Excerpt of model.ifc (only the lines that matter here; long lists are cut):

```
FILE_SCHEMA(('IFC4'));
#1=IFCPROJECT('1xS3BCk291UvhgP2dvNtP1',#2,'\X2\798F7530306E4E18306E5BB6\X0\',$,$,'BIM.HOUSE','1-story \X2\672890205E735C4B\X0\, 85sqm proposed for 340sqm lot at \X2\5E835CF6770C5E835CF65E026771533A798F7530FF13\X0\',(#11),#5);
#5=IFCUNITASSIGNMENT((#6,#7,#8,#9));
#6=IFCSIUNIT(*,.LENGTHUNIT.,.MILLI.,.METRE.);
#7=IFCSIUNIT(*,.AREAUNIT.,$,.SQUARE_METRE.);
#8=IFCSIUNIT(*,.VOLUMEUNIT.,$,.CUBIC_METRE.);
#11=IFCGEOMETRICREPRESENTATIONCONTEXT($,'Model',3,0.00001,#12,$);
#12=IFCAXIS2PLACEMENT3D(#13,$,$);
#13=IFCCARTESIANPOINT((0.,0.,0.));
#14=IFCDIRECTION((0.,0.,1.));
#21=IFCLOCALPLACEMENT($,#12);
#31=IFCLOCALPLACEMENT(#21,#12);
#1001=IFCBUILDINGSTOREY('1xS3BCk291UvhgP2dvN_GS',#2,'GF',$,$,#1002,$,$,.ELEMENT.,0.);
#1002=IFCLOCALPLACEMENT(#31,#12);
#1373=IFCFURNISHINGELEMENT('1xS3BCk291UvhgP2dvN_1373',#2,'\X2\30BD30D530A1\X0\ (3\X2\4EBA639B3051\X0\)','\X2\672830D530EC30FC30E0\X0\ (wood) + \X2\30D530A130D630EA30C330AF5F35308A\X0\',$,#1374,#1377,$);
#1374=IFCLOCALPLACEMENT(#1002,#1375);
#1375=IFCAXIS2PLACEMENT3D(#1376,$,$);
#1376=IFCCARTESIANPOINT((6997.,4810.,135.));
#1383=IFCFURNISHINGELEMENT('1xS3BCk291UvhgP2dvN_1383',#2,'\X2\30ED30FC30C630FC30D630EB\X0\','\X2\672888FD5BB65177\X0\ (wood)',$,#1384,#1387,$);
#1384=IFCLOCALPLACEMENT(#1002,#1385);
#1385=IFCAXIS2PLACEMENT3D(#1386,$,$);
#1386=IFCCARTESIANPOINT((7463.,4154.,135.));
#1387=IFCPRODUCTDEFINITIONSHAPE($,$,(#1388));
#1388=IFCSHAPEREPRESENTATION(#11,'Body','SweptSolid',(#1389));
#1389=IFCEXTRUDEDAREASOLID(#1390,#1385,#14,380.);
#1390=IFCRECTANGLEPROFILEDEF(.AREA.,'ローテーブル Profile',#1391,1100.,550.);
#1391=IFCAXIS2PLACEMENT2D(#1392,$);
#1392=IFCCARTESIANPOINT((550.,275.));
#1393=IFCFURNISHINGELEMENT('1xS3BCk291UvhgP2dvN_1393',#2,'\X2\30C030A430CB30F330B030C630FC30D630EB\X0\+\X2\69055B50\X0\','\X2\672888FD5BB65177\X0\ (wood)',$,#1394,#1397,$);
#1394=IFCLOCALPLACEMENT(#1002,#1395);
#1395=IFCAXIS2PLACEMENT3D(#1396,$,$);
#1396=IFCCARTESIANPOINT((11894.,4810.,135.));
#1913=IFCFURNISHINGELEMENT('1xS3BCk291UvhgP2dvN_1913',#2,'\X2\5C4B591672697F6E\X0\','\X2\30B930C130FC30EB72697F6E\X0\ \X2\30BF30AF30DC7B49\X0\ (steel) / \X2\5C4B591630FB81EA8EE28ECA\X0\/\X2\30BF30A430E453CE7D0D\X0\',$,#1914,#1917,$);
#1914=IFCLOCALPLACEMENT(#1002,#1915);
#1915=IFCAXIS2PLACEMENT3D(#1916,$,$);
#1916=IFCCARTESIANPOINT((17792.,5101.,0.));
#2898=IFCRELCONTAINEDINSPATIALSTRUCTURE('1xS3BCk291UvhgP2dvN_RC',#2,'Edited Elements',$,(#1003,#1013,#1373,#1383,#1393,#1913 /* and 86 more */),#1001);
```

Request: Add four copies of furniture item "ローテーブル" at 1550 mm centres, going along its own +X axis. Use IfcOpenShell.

```python
import ifcopenshell
import ifcopenshell.api.geometry
import ifcopenshell.api.root
import ifcopenshell.util.element
import ifcopenshell.util.placement
import ifcopenshell.util.unit

model = ifcopenshell.open("model.ifc")
unit_scale = ifcopenshell.util.unit.calculate_unit_scale(model)


def reuse_history(source, copy):
    """copy_class also copies each property set's owner history, people and application; keep the originals."""
    for rel in copy.IsDefinedBy:
        if rel.is_a("IfcRelDefinesByProperties") and (history := rel.RelatingPropertyDefinition.OwnerHistory):
            rel.RelatingPropertyDefinition.OwnerHistory = source.OwnerHistory
            ifcopenshell.util.element.remove_deep2(model, history)


source = model.by_id(1383)
base = ifcopenshell.util.placement.get_local_placement(source.ObjectPlacement)
step = base[:3, 0] * 1.55 / unit_scale

for i in range(1, 5):
    copy = ifcopenshell.api.root.copy_class(model, product=source)
    copy.Representation = ifcopenshell.util.element.copy_deep(
        model, source.Representation, exclude=["IfcGeometricRepresentationContext", "IfcRepresentationMap"]
    )
    reuse_history(source, copy)
    matrix = base.copy()
    matrix[:3, 3] += i * step
    print("added at", matrix[:3, 3].round(3) + 0.0)
    ifcopenshell.api.geometry.edit_object_placement(model, product=copy, matrix=matrix, is_si=False)

model.write("model_updated.ifc")
```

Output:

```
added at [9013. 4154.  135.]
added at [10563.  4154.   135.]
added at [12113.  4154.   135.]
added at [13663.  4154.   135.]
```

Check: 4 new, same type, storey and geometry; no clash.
